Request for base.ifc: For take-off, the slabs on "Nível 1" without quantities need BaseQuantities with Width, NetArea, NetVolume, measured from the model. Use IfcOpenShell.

First a look at what the model holds.

```python
import ifcopenshell
import ifcopenshell.util.element
import ifcopenshell.util.unit

model = ifcopenshell.open("base.ifc")
print(model.schema)
for unit_type in ("LENGTHUNIT", "AREAUNIT", "VOLUMEUNIT"):
    print(unit_type, ifcopenshell.util.unit.calculate_unit_scale(model, unit_type))
storey = next(s for s in model.by_type("IfcBuildingStorey") if s.Name == "Nível 1")
slabs = [e for e in ifcopenshell.util.element.get_decomposition(storey) if e.is_a("IfcSlab")]
for e in sorted(slabs, key=lambda e: e.id()):
    print(e.id(), e.is_a(), e.Name, list(ifcopenshell.util.element.get_psets(e, qtos_only=True)), sep=" | ")
```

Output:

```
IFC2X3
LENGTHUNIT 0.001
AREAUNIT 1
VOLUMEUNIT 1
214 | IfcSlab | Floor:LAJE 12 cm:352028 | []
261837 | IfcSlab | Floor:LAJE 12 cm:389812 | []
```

```python
import ifcopenshell
import ifcopenshell.api.pset
import ifcopenshell.geom
import ifcopenshell.util.element
import ifcopenshell.util.shape
import ifcopenshell.util.unit

model = ifcopenshell.open("base.ifc")
unit_scale = ifcopenshell.util.unit.calculate_unit_scale(model)
area_scale = ifcopenshell.util.unit.calculate_unit_scale(model, "AREAUNIT")
volume_scale = ifcopenshell.util.unit.calculate_unit_scale(model, "VOLUMEUNIT")
settings = ifcopenshell.geom.settings()

storey = next(s for s in model.by_type("IfcBuildingStorey") if s.Name == "Nível 1")
slabs = [e for e in ifcopenshell.util.element.get_decomposition(storey) if e.is_a("IfcSlab")]

for e in sorted(slabs, key=lambda e: e.id()):
    if ifcopenshell.util.element.get_psets(e, qtos_only=True, should_inherit=False):
        continue
    # Geometry comes back in metres, in the element's own axes.
    shape = ifcopenshell.geom.create_shape(settings, e)
    values = {
        "Width": ifcopenshell.util.shape.get_z(shape.geometry) / unit_scale,
        "NetArea": ifcopenshell.util.shape.get_footprint_area(shape.geometry) / area_scale,
        "NetVolume": ifcopenshell.util.shape.get_volume(shape.geometry) / volume_scale,
    }
    qto = ifcopenshell.api.pset.add_qto(model, product=e, name="BaseQuantities")
    ifcopenshell.api.pset.edit_qto(model, qto=qto, properties=values)
    print(e.id(), {k: round(v, 3) for k, v in values.items()})

model.write("base_updated.ifc")
```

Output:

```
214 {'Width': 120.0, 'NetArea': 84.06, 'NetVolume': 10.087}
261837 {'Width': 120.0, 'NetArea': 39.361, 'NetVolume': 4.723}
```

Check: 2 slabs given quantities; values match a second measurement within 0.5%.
